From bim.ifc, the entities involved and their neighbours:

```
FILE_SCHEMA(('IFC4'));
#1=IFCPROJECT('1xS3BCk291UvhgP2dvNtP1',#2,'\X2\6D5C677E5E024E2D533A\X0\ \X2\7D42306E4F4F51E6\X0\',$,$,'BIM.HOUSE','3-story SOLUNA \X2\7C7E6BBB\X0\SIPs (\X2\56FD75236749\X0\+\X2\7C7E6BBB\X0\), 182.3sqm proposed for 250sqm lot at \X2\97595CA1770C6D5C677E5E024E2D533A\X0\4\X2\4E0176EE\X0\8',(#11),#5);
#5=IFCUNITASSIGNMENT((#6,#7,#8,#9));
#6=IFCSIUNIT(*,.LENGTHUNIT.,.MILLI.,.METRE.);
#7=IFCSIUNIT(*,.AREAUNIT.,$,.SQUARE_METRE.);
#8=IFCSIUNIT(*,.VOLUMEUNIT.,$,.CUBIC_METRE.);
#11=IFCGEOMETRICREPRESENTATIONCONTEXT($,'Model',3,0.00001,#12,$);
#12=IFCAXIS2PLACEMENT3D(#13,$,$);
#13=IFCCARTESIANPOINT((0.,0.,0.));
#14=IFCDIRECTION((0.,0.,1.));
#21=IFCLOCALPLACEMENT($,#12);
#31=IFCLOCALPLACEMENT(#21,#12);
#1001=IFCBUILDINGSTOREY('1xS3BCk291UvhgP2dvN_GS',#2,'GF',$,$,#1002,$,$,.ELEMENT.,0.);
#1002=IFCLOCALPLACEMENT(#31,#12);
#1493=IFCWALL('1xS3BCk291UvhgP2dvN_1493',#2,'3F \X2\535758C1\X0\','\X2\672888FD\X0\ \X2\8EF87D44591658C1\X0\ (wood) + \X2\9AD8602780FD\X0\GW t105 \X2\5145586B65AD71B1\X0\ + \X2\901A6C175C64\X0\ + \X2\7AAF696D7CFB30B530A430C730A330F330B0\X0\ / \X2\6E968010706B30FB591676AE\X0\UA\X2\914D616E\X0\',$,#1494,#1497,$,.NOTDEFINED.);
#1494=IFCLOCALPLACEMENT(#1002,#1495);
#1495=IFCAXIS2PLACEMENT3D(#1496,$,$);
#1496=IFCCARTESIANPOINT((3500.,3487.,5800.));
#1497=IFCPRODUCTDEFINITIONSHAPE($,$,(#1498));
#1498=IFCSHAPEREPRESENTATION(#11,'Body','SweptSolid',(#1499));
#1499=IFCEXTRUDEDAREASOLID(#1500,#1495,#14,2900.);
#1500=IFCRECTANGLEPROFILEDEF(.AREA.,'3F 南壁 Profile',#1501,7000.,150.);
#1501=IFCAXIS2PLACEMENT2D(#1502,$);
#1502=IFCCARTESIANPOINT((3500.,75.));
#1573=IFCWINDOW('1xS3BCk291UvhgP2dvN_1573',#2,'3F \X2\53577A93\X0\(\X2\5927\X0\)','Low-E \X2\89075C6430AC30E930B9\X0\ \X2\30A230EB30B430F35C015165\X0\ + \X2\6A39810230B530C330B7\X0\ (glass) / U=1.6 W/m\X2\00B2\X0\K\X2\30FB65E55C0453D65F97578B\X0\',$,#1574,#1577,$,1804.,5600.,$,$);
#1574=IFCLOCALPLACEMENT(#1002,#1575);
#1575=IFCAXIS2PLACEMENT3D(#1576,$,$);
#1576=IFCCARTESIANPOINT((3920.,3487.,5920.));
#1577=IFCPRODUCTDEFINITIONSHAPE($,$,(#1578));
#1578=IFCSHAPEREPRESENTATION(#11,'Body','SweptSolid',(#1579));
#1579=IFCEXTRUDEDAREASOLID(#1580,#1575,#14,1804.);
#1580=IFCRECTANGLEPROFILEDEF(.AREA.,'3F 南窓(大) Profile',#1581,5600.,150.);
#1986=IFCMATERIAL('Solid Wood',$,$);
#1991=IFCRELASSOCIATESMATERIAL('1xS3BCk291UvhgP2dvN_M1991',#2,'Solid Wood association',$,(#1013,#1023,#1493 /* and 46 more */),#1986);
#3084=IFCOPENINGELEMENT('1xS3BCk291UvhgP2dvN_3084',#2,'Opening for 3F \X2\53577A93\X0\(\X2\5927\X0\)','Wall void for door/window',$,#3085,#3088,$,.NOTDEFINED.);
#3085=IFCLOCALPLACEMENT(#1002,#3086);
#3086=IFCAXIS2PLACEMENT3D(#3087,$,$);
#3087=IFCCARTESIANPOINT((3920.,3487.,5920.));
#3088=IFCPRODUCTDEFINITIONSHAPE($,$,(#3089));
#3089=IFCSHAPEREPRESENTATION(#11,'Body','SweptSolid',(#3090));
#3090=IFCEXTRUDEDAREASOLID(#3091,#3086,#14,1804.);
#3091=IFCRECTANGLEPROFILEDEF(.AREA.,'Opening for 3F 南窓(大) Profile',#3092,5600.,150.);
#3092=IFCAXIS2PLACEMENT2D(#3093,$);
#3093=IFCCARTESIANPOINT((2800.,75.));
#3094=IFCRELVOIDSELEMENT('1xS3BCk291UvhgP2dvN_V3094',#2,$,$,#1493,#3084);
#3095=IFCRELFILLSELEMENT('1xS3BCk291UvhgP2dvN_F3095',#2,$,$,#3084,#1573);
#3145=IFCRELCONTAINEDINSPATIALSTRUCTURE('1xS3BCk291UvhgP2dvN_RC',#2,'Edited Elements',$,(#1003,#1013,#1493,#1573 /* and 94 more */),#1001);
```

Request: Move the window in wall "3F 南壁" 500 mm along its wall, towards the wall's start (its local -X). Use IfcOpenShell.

```python
import ifcopenshell
import ifcopenshell.api.geometry
import ifcopenshell.util.placement
import ifcopenshell.util.unit

model = ifcopenshell.open("bim.ifc")
unit_scale = ifcopenshell.util.unit.calculate_unit_scale(model)

window = model.by_guid("1xS3BCk291UvhgP2dvN_1573")
opening = window.FillsVoids[0].RelatingOpeningElement
wall = opening.VoidsElements[0].RelatingBuildingElement

wall_matrix = ifcopenshell.util.placement.get_local_placement(wall.ObjectPlacement)
shift = wall_matrix[:3, 0] * -0.5 / unit_scale
before = ifcopenshell.util.placement.get_local_placement(window.ObjectPlacement)[:3, 3].copy()

# The window is not placed relative to its opening, so move both.
for product in (opening, window):
    matrix = ifcopenshell.util.placement.get_local_placement(product.ObjectPlacement)
    matrix[:3, 3] += shift
    ifcopenshell.api.geometry.edit_object_placement(model, product=product, matrix=matrix, is_si=False)

after = ifcopenshell.util.placement.get_local_placement(window.ObjectPlacement)[:3, 3]
print("window moved by", (after - before).round(3) + 0.0)

model.write("bim_v2.ifc")
```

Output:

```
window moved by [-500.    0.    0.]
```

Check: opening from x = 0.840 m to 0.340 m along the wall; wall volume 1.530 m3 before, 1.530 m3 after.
